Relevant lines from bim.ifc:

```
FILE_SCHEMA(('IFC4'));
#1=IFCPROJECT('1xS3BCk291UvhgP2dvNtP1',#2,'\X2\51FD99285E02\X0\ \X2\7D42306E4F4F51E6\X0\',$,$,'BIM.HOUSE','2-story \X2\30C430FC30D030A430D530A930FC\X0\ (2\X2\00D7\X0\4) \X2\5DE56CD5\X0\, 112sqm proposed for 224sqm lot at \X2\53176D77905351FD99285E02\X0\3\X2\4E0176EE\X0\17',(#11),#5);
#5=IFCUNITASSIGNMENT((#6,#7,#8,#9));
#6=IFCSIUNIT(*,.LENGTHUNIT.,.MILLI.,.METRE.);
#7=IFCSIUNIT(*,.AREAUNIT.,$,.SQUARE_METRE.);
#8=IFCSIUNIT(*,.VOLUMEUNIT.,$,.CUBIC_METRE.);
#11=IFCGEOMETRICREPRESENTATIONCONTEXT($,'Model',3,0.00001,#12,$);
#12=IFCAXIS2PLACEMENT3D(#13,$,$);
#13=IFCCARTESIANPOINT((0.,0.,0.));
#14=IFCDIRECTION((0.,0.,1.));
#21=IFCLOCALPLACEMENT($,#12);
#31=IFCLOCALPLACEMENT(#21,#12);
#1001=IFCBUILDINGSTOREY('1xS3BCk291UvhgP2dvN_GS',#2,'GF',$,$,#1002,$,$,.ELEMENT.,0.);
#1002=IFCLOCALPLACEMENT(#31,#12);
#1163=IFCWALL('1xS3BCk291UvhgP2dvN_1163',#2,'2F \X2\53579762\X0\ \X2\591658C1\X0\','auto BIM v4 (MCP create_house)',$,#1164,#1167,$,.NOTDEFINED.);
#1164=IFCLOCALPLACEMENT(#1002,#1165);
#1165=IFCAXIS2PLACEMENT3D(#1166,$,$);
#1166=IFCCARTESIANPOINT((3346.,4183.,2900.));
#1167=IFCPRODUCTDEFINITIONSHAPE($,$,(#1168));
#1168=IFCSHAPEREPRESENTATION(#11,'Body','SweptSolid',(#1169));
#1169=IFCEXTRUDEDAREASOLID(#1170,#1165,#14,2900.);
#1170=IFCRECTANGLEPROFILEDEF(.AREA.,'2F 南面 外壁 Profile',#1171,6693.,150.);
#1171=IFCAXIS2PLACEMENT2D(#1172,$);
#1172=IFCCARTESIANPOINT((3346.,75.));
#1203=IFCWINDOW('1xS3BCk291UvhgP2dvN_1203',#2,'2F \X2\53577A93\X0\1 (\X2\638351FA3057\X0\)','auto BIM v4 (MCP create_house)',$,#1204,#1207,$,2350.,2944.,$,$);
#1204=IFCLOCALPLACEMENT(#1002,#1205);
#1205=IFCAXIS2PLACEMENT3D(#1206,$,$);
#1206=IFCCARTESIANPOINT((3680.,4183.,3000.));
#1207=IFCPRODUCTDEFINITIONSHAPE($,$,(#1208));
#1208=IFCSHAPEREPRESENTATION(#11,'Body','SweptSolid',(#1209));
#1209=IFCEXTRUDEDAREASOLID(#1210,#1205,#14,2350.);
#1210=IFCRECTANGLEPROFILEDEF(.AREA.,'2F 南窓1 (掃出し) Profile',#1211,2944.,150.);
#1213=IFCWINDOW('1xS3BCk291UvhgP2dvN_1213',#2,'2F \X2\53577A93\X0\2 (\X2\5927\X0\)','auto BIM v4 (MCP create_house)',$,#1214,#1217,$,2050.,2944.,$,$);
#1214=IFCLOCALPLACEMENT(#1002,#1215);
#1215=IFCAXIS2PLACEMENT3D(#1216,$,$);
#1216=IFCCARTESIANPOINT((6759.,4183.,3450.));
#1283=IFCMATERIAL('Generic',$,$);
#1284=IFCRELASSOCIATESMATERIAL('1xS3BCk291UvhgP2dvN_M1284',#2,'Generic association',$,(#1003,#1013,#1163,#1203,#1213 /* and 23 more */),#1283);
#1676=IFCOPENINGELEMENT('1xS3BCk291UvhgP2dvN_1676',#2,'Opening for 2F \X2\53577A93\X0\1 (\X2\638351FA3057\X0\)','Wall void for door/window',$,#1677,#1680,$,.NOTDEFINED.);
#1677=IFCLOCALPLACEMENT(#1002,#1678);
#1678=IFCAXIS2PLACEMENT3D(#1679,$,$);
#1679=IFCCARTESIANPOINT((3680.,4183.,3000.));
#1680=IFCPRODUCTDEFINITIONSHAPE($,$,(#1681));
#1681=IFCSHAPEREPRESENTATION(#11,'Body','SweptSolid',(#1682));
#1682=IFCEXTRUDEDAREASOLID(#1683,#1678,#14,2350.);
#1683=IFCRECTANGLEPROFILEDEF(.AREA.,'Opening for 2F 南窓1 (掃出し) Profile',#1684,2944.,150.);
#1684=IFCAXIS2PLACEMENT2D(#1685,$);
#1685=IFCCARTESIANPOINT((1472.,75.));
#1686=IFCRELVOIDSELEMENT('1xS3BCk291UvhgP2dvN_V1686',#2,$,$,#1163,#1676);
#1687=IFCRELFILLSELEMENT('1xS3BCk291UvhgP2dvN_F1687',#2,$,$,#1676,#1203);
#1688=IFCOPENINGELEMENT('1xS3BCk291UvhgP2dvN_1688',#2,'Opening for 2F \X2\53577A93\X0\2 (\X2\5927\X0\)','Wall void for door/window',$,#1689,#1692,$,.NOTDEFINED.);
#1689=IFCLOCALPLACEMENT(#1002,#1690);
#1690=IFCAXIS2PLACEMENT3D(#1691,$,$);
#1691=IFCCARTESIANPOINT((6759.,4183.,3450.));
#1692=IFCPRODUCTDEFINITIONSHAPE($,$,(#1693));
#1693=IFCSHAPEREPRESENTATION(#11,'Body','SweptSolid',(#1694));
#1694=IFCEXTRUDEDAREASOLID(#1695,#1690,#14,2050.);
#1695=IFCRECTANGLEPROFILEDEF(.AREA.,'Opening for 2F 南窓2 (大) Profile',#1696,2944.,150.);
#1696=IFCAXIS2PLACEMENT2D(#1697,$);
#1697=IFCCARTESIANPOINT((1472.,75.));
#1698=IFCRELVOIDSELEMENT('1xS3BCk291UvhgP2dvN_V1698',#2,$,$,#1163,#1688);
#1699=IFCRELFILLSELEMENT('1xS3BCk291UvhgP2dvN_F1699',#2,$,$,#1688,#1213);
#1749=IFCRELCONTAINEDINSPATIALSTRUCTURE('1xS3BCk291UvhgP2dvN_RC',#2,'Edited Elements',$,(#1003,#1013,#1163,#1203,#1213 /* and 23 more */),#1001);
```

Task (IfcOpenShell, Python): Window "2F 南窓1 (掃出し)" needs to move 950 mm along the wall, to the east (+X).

```python
import ifcopenshell
import ifcopenshell.api.geometry
import ifcopenshell.util.placement
import ifcopenshell.util.unit

model = ifcopenshell.open("bim.ifc")
unit_scale = ifcopenshell.util.unit.calculate_unit_scale(model)

window = model.by_id(1203)
opening = window.FillsVoids[0].RelatingOpeningElement
wall = opening.VoidsElements[0].RelatingBuildingElement

wall_matrix = ifcopenshell.util.placement.get_local_placement(wall.ObjectPlacement)
shift = wall_matrix[:3, 0] * 0.95 / unit_scale
before = ifcopenshell.util.placement.get_local_placement(window.ObjectPlacement)[:3, 3].copy()

# The window is not placed relative to its opening, so move both.
for product in (opening, window):
    matrix = ifcopenshell.util.placement.get_local_placement(product.ObjectPlacement)
    matrix[:3, 3] += shift
    ifcopenshell.api.geometry.edit_object_placement(model, product=product, matrix=matrix, is_si=False)

after = ifcopenshell.util.placement.get_local_placement(window.ObjectPlacement)[:3, 3]
print("window moved by", (after - before).round(3) + 0.0)

model.write("bim-out.ifc")
```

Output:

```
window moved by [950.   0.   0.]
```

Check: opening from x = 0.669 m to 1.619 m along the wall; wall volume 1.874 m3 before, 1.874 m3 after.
